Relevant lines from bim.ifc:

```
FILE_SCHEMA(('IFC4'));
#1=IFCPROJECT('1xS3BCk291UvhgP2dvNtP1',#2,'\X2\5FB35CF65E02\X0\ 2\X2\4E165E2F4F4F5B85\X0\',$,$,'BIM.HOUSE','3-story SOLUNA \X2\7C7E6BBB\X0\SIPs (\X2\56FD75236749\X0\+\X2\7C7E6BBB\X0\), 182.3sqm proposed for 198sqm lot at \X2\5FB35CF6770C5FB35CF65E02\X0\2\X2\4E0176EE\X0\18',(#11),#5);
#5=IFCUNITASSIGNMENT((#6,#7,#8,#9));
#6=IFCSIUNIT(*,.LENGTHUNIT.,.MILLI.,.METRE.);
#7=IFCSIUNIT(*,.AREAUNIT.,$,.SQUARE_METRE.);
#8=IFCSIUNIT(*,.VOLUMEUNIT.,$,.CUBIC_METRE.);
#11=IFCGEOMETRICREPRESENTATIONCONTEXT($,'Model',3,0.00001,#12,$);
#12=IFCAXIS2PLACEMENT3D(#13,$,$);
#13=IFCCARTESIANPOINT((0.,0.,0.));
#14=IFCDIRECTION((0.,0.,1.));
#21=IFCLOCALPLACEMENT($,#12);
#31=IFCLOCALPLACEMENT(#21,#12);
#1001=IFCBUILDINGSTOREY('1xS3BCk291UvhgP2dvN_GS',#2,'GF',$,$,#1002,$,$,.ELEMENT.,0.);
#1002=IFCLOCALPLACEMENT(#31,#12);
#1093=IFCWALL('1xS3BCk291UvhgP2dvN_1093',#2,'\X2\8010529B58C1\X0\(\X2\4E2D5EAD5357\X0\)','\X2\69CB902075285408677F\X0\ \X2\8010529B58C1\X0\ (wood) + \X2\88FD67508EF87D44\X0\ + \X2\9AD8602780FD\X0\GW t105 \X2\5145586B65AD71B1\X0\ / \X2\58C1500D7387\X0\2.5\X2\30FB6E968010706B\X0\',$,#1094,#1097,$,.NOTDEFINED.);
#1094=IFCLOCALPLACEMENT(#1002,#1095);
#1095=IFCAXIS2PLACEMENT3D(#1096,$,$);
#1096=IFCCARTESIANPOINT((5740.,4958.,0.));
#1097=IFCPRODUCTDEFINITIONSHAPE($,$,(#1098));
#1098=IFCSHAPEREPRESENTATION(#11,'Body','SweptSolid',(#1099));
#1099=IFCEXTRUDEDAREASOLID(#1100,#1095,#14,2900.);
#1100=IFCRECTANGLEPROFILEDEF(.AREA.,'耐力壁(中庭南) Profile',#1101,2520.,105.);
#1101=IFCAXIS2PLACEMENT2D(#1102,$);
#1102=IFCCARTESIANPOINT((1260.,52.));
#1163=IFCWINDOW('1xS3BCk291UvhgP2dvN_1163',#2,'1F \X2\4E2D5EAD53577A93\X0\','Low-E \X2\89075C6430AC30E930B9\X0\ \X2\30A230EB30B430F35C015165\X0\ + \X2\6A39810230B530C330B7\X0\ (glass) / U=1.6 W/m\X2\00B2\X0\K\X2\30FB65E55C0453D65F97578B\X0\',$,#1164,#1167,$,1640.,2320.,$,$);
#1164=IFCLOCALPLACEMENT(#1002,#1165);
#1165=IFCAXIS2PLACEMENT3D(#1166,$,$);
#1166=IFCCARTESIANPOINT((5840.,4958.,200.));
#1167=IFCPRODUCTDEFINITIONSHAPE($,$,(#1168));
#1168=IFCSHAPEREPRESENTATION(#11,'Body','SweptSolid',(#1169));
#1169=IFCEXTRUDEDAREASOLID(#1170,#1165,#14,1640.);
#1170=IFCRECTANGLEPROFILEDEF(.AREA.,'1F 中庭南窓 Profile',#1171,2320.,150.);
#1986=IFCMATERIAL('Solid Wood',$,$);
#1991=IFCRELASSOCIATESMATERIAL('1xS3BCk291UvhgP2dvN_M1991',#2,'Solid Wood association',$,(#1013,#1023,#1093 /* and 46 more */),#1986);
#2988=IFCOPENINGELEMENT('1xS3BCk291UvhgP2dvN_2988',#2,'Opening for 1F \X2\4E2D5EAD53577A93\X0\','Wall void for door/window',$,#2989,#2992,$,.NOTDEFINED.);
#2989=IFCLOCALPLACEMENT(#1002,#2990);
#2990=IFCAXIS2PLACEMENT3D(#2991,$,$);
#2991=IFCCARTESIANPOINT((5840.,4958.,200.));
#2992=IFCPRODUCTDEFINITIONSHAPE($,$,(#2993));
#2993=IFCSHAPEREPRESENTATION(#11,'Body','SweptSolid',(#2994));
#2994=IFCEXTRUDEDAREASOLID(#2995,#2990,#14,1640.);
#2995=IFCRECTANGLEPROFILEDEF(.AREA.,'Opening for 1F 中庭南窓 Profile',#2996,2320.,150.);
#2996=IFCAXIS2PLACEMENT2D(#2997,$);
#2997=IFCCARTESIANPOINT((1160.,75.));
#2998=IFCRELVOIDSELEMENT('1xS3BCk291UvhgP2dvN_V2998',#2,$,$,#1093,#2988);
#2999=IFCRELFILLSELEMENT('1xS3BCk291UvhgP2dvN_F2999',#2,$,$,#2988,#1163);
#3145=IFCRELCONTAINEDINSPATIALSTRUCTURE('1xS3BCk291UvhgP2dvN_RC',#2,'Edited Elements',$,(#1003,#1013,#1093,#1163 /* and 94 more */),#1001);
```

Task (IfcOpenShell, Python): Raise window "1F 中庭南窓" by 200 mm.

```python
import numpy as np
import ifcopenshell
import ifcopenshell.api.geometry
import ifcopenshell.util.placement
import ifcopenshell.util.unit

model = ifcopenshell.open("bim.ifc")
unit_scale = ifcopenshell.util.unit.calculate_unit_scale(model)

window = model.by_guid("1xS3BCk291UvhgP2dvN_1163")
opening = window.FillsVoids[0].RelatingOpeningElement
dz = 200.0

shift = np.array([0.0, 0.0, dz])
# The window is not placed relative to its opening, so move both.
for product in (opening, window):
    matrix = ifcopenshell.util.placement.get_local_placement(product.ObjectPlacement)
    matrix[:3, 3] += shift
    ifcopenshell.api.geometry.edit_object_placement(model, product=product, matrix=matrix, is_si=False)

print(f"moved by {dz * unit_scale:+.3f} m")

model.write("bim_v2.ifc")
```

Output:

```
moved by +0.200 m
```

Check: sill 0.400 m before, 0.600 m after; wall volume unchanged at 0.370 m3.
